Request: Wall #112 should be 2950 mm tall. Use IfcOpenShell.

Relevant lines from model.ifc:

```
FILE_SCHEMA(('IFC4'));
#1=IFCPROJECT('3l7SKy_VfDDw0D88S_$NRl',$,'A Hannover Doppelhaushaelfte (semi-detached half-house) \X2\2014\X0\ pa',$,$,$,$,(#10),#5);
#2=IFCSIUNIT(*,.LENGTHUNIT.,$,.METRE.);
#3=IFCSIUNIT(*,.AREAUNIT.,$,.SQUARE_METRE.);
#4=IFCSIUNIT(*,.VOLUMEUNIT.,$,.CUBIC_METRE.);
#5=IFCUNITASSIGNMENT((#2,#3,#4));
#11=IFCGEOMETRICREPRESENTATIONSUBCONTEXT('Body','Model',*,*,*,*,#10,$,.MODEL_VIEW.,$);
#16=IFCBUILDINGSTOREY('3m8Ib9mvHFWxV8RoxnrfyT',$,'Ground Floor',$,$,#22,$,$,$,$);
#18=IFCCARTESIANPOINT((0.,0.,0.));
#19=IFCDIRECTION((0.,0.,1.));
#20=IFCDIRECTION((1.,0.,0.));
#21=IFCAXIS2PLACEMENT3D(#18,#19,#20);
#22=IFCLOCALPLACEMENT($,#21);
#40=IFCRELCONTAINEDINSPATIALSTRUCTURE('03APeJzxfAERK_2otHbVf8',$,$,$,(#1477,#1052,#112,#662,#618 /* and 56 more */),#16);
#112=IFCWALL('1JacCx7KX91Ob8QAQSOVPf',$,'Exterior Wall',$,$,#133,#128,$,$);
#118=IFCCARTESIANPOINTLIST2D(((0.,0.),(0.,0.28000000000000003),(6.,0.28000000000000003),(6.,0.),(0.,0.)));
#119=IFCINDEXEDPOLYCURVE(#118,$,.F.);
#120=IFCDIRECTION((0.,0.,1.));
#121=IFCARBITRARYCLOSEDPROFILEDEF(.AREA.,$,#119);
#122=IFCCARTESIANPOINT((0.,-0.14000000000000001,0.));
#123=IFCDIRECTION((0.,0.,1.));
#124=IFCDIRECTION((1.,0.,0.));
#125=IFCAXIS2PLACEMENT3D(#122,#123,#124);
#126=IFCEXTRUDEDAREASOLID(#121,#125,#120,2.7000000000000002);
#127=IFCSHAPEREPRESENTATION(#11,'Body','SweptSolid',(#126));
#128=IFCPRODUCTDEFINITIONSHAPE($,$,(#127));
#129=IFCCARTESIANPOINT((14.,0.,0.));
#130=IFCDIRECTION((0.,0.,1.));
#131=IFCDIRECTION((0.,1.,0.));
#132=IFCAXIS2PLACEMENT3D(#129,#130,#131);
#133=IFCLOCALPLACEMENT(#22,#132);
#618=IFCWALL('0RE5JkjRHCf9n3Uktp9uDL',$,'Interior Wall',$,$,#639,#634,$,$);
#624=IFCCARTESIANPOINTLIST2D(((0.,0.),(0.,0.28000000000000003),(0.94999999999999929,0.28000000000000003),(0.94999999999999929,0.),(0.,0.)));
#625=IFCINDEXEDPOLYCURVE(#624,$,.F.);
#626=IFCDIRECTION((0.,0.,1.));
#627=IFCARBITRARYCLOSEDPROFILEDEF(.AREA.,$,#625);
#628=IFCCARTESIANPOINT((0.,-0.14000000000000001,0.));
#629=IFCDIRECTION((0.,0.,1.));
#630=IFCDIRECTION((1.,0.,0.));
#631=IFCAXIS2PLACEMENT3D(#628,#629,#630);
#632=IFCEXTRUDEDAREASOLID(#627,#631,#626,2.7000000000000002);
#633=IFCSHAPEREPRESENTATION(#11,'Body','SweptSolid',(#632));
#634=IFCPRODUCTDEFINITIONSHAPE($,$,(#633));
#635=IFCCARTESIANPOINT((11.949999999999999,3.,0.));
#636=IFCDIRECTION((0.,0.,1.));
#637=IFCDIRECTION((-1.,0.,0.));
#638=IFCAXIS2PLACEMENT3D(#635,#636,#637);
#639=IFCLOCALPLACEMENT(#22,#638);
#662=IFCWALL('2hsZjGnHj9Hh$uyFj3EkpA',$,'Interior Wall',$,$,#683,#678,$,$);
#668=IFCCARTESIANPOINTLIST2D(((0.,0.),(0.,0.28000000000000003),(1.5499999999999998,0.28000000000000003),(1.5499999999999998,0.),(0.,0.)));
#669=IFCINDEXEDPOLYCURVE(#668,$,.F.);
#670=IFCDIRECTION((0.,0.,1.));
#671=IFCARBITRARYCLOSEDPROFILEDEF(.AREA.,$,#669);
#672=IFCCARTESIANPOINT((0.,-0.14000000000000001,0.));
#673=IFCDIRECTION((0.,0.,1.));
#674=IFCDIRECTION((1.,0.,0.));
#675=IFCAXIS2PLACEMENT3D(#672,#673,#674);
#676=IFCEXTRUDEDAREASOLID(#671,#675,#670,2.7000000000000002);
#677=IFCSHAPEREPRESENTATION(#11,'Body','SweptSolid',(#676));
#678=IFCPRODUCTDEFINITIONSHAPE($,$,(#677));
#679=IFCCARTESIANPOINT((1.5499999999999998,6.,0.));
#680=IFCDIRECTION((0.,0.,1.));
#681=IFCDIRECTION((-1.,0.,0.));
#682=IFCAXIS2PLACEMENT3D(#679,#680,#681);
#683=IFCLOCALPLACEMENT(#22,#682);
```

```python
import ifcopenshell
import ifcopenshell.geom
import ifcopenshell.util.representation
import ifcopenshell.util.shape

model = ifcopenshell.open("model.ifc")
settings = ifcopenshell.geom.settings()


def volume(element):
    """Net volume in cubic metres, openings subtracted."""
    shape = ifcopenshell.geom.create_shape(settings, element)
    return ifcopenshell.util.shape.get_volume(shape.geometry)


wall = model.by_id(112)
before = volume(wall)

body = ifcopenshell.util.representation.get_representation(wall, "Model", "Body")
solid = body.Items[0]
old_height = solid.Depth
solid.Depth = 2.95
after = volume(wall)

print(f"height {old_height:g} -> {solid.Depth:g}, volume {before:.3f} -> {after:.3f} m3")

model.write("model_v2.ifc")
```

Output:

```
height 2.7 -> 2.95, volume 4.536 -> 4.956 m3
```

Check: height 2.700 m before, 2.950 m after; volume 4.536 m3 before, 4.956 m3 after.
